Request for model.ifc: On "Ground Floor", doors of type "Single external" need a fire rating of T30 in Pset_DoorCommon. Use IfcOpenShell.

First a look at what the model holds.

```python
import ifcopenshell
import ifcopenshell.util.element

model = ifcopenshell.open("model.ifc")
print(model.schema)
storey = next(s for s in model.by_type("IfcBuildingStorey") if s.Name == "Ground Floor")
doors = [e for e in ifcopenshell.util.element.get_decomposition(storey) if e.is_a("IfcDoor")]
seen = {}
for e in doors:
    element_type = ifcopenshell.util.element.get_type(e)
    key = (element_type.Name if element_type != e and element_type else None, ifcopenshell.util.element.get_pset(e, "Pset_DoorCommon", "FireRating"))
    seen[key] = seen.get(key, 0) + 1
for (name, value), count in sorted(seen.items(), key=str):
    print(count, "x", name, "|", value)
```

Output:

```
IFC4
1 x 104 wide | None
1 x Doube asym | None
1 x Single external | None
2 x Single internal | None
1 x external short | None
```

```python
import ifcopenshell
import ifcopenshell.api.pset
import ifcopenshell.util.element

model = ifcopenshell.open("model.ifc")

storey = next(s for s in model.by_type("IfcBuildingStorey") if s.Name == "Ground Floor")
doors = [e for e in ifcopenshell.util.element.get_decomposition(storey) if e.is_a("IfcDoor")]

count = 0
for e in doors:
    element_type = ifcopenshell.util.element.get_type(e)
    if element_type in (None, e) or element_type.Name != "Single external":
        continue
    # add_pset returns the element's existing set when there is one.
    pset = ifcopenshell.api.pset.add_pset(model, product=e, name="Pset_DoorCommon")
    ifcopenshell.api.pset.edit_pset(model, pset=pset, properties={"FireRating": "T30"})
    count += 1

print(count, "doors updated")

model.write("model_v2.ifc")
```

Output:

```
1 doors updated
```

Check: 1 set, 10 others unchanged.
